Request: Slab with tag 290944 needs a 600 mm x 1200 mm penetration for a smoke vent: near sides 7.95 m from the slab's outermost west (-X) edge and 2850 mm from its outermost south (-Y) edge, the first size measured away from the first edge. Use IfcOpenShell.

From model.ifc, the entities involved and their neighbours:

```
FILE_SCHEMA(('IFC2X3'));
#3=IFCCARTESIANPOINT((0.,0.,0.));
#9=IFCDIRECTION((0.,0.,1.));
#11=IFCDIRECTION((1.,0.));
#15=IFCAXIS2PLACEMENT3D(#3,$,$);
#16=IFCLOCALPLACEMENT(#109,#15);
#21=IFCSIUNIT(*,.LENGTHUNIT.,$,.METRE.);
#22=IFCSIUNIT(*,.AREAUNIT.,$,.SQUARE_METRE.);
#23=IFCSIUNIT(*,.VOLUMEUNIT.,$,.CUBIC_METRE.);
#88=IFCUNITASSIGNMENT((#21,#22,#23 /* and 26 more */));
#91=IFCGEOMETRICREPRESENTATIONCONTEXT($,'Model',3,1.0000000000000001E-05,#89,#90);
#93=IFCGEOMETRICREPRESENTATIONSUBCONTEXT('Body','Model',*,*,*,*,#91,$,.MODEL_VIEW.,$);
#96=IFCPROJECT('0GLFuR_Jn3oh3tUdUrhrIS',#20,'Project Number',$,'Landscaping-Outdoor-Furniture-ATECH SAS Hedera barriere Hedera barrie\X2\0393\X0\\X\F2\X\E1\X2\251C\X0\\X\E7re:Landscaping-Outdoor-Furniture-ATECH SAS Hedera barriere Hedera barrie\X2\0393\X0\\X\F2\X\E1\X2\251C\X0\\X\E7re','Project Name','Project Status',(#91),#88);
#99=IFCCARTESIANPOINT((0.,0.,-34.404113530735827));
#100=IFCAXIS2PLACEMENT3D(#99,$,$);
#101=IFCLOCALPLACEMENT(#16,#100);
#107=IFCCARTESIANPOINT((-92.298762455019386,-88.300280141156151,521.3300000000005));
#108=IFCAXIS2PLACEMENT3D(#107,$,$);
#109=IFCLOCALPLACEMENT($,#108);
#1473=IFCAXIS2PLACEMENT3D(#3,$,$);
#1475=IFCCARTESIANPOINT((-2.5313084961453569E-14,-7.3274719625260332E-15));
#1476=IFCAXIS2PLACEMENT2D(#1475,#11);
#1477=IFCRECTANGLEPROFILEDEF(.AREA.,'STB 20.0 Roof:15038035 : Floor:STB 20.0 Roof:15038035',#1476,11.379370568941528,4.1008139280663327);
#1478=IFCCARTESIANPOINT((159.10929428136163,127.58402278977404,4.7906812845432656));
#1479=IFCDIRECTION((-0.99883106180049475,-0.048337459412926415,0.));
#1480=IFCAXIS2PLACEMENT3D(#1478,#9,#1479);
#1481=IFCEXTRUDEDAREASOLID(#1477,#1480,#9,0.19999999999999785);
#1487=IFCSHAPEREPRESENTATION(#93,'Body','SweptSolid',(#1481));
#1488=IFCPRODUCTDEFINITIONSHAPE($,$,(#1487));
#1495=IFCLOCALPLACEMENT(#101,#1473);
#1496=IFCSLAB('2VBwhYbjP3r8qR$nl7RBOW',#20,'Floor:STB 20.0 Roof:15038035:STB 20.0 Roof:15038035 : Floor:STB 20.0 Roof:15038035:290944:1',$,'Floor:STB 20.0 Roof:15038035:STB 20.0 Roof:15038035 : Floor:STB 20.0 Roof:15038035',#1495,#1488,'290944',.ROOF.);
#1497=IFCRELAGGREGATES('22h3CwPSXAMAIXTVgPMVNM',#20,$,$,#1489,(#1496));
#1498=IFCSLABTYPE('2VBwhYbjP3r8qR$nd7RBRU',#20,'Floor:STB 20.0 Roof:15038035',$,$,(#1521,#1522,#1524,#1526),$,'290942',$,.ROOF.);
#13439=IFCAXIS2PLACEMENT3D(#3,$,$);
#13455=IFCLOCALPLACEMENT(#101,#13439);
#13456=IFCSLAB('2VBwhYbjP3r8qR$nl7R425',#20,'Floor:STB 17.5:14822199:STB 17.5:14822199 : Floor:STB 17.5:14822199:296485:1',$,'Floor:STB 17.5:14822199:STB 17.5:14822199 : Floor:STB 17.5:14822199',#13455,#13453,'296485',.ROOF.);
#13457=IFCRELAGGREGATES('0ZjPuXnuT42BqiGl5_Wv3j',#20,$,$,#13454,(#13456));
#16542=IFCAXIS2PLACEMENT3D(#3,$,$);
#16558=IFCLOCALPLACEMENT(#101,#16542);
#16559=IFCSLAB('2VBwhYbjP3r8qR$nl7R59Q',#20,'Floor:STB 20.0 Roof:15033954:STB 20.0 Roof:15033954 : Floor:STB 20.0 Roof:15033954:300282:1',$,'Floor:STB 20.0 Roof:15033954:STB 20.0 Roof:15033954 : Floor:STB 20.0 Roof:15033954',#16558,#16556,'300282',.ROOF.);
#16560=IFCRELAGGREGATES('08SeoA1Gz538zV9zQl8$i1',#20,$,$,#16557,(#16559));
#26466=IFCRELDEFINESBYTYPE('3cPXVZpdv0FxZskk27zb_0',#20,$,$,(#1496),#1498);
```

```python
import numpy as np
import ifcopenshell
import ifcopenshell.api.feature
import ifcopenshell.api.geometry
import ifcopenshell.api.root
import ifcopenshell.geom
import ifcopenshell.util.placement
import ifcopenshell.util.representation
import ifcopenshell.util.shape
import ifcopenshell.util.unit

model = ifcopenshell.open("model.ifc")
unit_scale = ifcopenshell.util.unit.calculate_unit_scale(model)
settings = ifcopenshell.geom.settings()


def volume(element):
    """Net volume in cubic metres, openings subtracted."""
    shape = ifcopenshell.geom.create_shape(settings, element)
    return ifcopenshell.util.shape.get_volume(shape.geometry)


slab = model.by_id(1496)
before = volume(slab)

# Extent in the slab's own axes, in metres. The edges named are its -X and -Y sides.
slab_shape = ifcopenshell.geom.create_shape(settings, slab)
vertices = ifcopenshell.util.shape.get_vertices(slab_shape.geometry)
x_min, y_min, bottom = vertices.min(axis=0)
top = vertices[:, 2].max()

opening = ifcopenshell.api.root.create_entity(model, ifc_class="IfcOpeningElement", name="Smoke vent opening")
context = ifcopenshell.util.representation.get_context(model, "Model", "Body", "MODEL_VIEW")
width, depth = 0.6, 1.2
outline = [(0.0, 0.0), (width, 0.0), (width, depth), (0.0, depth), (0.0, 0.0)]
# Overshoot both faces by 50 mm so the cut is clean.
shape = ifcopenshell.api.geometry.add_slab_representation(
    model, context=context, depth=top - bottom + 0.1, polyline=outline
)
ifcopenshell.api.geometry.assign_representation(model, product=opening, representation=shape)

matrix = ifcopenshell.util.placement.get_local_placement(slab.ObjectPlacement)
matrix[:, 3] = matrix @ np.append(np.array([x_min + 7.95, y_min + 2.85, bottom - 0.05]) / unit_scale, 1.0)
ifcopenshell.api.geometry.edit_object_placement(model, product=opening, matrix=matrix, is_si=False)
ifcopenshell.api.feature.add_feature(model, feature=opening, element=slab)

after = volume(slab)

print(f"slab volume {before:.3f} -> {after:.3f} m3")

model.write("model_updated.ifc")
```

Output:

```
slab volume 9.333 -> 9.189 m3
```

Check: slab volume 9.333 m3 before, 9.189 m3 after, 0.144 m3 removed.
